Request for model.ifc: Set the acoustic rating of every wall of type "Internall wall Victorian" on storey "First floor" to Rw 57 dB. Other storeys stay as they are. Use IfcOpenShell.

First a look at what the model holds.

```python
import ifcopenshell
import ifcopenshell.util.element

model = ifcopenshell.open("model.ifc")
print(model.schema)
storey = next(s for s in model.by_type("IfcBuildingStorey") if s.Name == "First floor")
walls = [e for e in ifcopenshell.util.element.get_decomposition(storey) if e.is_a("IfcWall")]
seen = {}
for e in walls:
    element_type = ifcopenshell.util.element.get_type(e)
    key = (element_type.Name if element_type != e and element_type else None, ifcopenshell.util.element.get_pset(e, "Pset_WallCommon", "AcousticRating"))
    seen[key] = seen.get(key, 0) + 1
for (name, value), count in sorted(seen.items(), key=str):
    print(count, "x", name, "|", value)
```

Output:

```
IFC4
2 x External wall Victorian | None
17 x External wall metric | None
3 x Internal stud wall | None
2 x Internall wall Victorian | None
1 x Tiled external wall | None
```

```python
import ifcopenshell
import ifcopenshell.api.pset
import ifcopenshell.util.element

model = ifcopenshell.open("model.ifc")

storey = next(s for s in model.by_type("IfcBuildingStorey") if s.Name == "First floor")
walls = [e for e in ifcopenshell.util.element.get_decomposition(storey) if e.is_a("IfcWall")]

count = 0
for e in walls:
    element_type = ifcopenshell.util.element.get_type(e)
    if element_type in (None, e) or element_type.Name != "Internall wall Victorian":
        continue
    # add_pset returns the element's existing set when there is one.
    pset = ifcopenshell.api.pset.add_pset(model, product=e, name="Pset_WallCommon")
    ifcopenshell.api.pset.edit_pset(model, pset=pset, properties={"AcousticRating": "Rw 57 dB"})
    count += 1

print(count, "walls updated")

model.write("model_v2.ifc")
```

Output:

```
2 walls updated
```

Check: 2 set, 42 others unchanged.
